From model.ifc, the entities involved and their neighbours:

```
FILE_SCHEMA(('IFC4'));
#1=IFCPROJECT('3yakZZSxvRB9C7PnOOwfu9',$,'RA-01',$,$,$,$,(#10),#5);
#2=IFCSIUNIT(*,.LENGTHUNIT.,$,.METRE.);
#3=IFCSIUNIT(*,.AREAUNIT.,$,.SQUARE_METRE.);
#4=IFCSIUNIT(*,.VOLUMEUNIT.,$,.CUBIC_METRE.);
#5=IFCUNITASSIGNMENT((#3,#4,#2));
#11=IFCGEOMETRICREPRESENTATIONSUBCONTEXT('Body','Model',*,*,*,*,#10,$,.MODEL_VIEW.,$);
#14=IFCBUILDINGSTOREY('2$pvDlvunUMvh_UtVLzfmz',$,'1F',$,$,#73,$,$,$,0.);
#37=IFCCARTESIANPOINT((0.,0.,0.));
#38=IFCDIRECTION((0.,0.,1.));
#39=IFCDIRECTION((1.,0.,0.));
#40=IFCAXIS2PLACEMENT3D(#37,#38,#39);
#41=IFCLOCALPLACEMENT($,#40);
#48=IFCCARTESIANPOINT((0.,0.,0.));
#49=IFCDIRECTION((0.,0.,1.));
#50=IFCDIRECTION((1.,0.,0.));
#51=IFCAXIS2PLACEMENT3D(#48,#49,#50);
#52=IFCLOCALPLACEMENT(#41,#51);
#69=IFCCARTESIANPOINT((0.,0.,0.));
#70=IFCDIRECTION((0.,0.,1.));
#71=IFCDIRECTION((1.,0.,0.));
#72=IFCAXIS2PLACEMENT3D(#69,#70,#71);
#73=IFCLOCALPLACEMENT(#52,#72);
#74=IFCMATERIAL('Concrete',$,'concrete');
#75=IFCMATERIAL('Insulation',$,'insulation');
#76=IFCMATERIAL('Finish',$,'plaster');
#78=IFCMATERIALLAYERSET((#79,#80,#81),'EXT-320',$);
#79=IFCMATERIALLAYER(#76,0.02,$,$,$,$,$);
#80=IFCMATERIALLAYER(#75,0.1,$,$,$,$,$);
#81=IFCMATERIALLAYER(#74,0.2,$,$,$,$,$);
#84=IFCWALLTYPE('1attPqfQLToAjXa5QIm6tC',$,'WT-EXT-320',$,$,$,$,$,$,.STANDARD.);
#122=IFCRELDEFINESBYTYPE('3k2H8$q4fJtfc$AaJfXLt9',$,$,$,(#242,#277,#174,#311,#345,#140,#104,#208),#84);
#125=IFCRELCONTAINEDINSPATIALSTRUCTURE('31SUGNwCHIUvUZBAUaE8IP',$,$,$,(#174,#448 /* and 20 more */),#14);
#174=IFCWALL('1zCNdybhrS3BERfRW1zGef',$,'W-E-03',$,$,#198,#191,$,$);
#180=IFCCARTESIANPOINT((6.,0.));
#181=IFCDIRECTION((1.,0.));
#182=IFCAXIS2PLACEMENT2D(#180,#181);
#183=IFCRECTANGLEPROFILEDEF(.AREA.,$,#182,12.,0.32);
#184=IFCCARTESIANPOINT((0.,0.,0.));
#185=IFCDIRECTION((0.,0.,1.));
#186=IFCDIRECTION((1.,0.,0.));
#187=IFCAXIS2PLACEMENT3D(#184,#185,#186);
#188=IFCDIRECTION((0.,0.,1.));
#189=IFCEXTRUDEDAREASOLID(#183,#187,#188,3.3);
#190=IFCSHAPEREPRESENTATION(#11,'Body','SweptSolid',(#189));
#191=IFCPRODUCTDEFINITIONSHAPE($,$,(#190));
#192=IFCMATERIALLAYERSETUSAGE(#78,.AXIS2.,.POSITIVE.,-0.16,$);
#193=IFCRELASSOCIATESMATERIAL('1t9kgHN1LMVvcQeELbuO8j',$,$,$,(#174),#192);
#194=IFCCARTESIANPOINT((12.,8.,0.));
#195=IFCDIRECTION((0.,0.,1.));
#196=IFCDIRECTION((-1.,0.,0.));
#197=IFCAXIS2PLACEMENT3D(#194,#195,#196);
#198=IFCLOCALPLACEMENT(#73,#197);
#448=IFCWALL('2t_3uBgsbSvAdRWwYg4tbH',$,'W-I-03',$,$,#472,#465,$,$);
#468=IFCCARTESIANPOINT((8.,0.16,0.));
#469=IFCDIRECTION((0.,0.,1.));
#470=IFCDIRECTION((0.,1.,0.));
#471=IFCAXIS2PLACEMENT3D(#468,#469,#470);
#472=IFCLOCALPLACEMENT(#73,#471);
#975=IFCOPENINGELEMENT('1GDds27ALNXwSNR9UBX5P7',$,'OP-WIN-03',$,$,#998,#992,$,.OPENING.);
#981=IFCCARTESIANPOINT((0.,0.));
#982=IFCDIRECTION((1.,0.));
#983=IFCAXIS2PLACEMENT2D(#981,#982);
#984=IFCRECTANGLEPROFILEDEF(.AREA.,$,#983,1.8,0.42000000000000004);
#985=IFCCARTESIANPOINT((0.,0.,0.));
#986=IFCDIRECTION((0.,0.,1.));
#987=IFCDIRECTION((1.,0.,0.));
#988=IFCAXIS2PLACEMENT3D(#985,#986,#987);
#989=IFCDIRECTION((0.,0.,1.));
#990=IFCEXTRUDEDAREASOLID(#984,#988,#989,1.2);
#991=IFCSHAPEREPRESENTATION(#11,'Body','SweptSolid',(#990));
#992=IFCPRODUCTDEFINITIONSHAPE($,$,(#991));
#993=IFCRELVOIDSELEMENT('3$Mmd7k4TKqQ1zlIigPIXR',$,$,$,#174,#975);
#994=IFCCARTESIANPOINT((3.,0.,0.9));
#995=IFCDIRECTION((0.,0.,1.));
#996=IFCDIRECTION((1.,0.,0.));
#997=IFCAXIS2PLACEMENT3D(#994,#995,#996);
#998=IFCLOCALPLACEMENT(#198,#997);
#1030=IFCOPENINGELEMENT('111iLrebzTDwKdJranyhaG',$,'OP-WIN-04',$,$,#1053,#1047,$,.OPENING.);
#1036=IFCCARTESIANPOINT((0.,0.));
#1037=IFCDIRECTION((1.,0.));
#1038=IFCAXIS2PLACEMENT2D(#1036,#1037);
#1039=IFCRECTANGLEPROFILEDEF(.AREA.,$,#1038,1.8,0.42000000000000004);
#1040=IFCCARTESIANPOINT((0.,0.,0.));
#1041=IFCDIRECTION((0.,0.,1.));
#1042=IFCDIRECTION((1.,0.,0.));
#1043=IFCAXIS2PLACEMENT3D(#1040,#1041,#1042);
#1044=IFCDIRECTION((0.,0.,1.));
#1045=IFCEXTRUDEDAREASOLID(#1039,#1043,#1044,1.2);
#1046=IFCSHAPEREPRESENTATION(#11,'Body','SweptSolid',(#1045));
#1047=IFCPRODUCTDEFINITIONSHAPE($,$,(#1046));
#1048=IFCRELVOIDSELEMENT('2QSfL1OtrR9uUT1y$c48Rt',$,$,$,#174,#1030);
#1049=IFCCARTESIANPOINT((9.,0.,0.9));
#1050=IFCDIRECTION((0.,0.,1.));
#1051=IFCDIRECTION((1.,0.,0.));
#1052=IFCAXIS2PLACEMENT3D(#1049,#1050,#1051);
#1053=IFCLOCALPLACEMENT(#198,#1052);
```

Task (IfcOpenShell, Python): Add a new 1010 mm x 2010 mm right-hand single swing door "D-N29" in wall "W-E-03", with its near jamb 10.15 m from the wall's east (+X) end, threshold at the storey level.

```python
import numpy as np
import ifcopenshell
import ifcopenshell.api.feature
import ifcopenshell.api.geometry
import ifcopenshell.api.root
import ifcopenshell.api.spatial
import ifcopenshell.geom
import ifcopenshell.util.element
import ifcopenshell.util.placement
import ifcopenshell.util.representation
import ifcopenshell.util.shape
import ifcopenshell.util.unit

model = ifcopenshell.open("model.ifc")
unit_scale = ifcopenshell.util.unit.calculate_unit_scale(model)
settings = ifcopenshell.geom.settings()


def volume(element):
    """Net volume in cubic metres, openings subtracted."""
    shape = ifcopenshell.geom.create_shape(settings, element)
    return ifcopenshell.util.shape.get_volume(shape.geometry)


wall = model.by_id(174)
storey = ifcopenshell.util.element.get_container(wall, ifc_class="IfcBuildingStorey")
context = ifcopenshell.util.representation.get_context(model, "Model", "Body", "MODEL_VIEW")
before = volume(wall)

width, height, from_end, sill = 1.01, 2.01, 10.15, 0.0  # metres

# The wall runs along its own X axis, and the end named is its -X end.
wall_shape = ifcopenshell.geom.create_shape(settings, wall)
x, y, z = ifcopenshell.util.shape.get_vertices(wall_shape.geometry).T
start = x.min() + from_end
face, thickness = float(y.min()), float(y.max() - y.min())
wall_matrix = ifcopenshell.util.placement.get_local_placement(wall.ObjectPlacement)
level = ifcopenshell.util.placement.get_local_placement(storey.ObjectPlacement)[2, 3]


def in_wall(x, y):
    """Placement at x, y metres in the wall's axes, at sill height."""
    matrix = wall_matrix.copy()
    matrix[:, 3] = wall_matrix @ np.array([x / unit_scale, y / unit_scale, 0.0, 1.0])
    matrix[2, 3] = level + sill / unit_scale
    return matrix


# Opening: a box that overshoots both wall faces by 50 mm.
opening = ifcopenshell.api.root.create_entity(model, ifc_class="IfcOpeningElement", predefined_type="OPENING")
box = ifcopenshell.api.geometry.add_wall_representation(
    model, context=context, length=width, height=height, thickness=thickness + 0.1
)
ifcopenshell.api.geometry.assign_representation(model, product=opening, representation=box)
ifcopenshell.api.geometry.edit_object_placement(model, product=opening, matrix=in_wall(start, face - 0.05), is_si=False)
ifcopenshell.api.feature.add_feature(model, feature=opening, element=wall)

door = ifcopenshell.api.root.create_entity(model, ifc_class="IfcDoor", name="D-N29", predefined_type="DOOR")
door.OverallWidth, door.OverallHeight = width / unit_scale, height / unit_scale
door.OperationType = "SINGLE_SWING_RIGHT"
body = ifcopenshell.api.geometry.add_door_representation(
    model,
    context=context,
    overall_width=door.OverallWidth,
    overall_height=door.OverallHeight,
    operation_type="SINGLE_SWING_RIGHT",
    lining_properties={"LiningDepth": thickness / unit_scale, "ThresholdDepth": thickness / unit_scale},
)
ifcopenshell.api.geometry.assign_representation(model, product=door, representation=body)
ifcopenshell.api.spatial.assign_container(model, products=[door], relating_structure=storey)
ifcopenshell.api.feature.add_filling(model, opening=opening, element=door)

# The lining spans the wall, so the door starts at the wall face.
ifcopenshell.api.geometry.edit_object_placement(model, product=door, matrix=in_wall(start, face), is_si=False)

after = volume(wall)

print(f"wall volume {before:.3f} -> {after:.3f} m3")

model.write("model_edited.ifc")
```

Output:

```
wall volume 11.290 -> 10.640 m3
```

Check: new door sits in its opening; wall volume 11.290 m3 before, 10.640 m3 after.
